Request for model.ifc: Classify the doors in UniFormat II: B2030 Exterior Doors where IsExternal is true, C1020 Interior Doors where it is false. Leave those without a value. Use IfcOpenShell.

First a look at what the model holds.

```python
import ifcopenshell
import ifcopenshell.util.element

model = ifcopenshell.open("model.ifc")
print(model.schema)
print("classifications:", [c.Name for c in model.by_type("IfcClassification")])
values = [ifcopenshell.util.element.get_pset(e, "Pset_DoorCommon", "IsExternal") for e in model.by_type("IfcDoor")]
for value in (True, False, None):
    print("IsExternal", value, values.count(value))
```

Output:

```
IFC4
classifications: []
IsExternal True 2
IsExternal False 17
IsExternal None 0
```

```python
import ifcopenshell
import ifcopenshell.api.classification
import ifcopenshell.util.element

model = ifcopenshell.open("model.ifc")

system = ifcopenshell.api.classification.add_classification(model, classification="UniFormat II")

doors = model.by_type("IfcDoor")
external = {e: ifcopenshell.util.element.get_pset(e, "Pset_DoorCommon", "IsExternal") for e in doors}
for flag, code, name in ((True, "B2030", "Exterior Doors"), (False, "C1020", "Interior Doors")):
    products = [e for e in doors if external[e] is flag]
    ifcopenshell.api.classification.add_reference(
        model, products=products, classification=system, identification=code, name=name
    )
    print(code, len(products))

model.write("model_v2.ifc")
```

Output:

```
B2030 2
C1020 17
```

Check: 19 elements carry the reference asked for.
